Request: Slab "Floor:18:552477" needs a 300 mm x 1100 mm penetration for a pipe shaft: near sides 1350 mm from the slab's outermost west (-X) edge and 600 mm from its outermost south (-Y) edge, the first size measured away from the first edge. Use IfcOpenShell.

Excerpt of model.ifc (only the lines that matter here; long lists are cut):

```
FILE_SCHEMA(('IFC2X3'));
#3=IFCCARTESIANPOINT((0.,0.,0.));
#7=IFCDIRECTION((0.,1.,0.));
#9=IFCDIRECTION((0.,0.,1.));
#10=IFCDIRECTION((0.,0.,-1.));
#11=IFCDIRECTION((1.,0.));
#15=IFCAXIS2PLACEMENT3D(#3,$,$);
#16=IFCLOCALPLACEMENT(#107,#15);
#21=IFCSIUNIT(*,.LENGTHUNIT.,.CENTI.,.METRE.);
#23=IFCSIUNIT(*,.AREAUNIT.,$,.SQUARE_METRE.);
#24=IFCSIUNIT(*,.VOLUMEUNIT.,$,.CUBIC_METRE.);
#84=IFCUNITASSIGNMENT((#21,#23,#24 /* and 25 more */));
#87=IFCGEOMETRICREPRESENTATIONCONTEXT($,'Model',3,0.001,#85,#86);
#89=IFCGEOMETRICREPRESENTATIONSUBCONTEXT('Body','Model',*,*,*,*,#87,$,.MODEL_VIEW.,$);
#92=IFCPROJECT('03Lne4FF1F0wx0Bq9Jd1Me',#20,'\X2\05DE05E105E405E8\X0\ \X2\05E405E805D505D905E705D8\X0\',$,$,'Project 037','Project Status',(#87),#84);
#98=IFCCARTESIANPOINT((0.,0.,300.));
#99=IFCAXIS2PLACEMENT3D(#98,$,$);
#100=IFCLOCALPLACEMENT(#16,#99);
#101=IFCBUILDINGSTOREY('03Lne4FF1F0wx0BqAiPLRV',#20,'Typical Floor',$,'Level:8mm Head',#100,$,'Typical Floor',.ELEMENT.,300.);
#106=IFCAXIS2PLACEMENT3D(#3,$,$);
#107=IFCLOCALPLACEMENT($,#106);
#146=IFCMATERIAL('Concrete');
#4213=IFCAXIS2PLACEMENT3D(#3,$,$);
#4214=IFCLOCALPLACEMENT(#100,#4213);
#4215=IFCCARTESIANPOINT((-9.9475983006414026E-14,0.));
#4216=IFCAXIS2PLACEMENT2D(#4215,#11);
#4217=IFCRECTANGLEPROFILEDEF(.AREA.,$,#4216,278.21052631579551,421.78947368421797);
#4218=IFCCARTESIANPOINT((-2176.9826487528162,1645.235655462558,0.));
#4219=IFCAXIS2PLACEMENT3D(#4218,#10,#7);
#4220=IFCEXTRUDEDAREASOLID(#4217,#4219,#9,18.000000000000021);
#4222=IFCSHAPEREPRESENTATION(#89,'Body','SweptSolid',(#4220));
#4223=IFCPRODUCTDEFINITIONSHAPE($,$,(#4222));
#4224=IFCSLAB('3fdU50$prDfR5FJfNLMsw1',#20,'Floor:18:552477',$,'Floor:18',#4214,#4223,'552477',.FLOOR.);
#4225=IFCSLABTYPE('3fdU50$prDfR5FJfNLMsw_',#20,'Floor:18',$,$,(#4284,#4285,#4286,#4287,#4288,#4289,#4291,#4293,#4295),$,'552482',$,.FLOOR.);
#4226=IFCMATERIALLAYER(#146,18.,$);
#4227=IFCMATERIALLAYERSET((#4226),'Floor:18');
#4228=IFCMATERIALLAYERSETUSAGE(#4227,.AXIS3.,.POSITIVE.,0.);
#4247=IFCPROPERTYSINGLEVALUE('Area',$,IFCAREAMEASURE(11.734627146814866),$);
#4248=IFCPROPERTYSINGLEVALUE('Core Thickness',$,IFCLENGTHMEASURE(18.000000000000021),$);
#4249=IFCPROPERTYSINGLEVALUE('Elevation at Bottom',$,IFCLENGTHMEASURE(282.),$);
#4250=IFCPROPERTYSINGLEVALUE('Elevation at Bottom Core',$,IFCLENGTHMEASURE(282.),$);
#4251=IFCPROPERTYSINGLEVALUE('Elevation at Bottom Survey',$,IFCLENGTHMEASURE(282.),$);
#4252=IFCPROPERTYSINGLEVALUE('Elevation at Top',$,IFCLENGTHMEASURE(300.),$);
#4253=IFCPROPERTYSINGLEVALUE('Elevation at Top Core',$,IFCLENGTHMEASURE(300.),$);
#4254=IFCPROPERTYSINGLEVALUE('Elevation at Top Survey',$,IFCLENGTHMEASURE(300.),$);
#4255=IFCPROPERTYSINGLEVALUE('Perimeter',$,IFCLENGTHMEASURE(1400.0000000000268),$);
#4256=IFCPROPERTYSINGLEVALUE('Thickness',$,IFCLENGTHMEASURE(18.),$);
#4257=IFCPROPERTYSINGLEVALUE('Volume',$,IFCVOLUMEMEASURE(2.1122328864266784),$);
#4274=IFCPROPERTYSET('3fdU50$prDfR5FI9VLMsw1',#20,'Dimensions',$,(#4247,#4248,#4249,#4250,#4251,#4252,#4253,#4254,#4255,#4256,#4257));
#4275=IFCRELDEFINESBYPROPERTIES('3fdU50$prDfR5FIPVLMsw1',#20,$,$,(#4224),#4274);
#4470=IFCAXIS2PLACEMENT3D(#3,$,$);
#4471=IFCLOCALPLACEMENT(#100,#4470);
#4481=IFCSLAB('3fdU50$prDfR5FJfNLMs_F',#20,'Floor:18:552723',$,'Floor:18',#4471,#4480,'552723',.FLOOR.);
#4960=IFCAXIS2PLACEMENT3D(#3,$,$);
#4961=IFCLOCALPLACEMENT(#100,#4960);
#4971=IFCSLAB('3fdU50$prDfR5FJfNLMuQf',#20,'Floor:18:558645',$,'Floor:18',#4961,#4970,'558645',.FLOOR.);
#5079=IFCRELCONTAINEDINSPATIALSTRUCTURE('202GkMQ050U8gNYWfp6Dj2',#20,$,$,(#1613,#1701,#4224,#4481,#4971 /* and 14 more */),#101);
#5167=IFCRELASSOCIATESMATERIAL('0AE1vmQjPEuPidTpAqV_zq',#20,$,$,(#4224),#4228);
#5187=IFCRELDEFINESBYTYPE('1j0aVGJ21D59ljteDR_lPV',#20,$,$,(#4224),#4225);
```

```python
import numpy as np
import ifcopenshell
import ifcopenshell.api.feature
import ifcopenshell.api.geometry
import ifcopenshell.api.pset
import ifcopenshell.api.root
import ifcopenshell.geom
import ifcopenshell.util.element
import ifcopenshell.util.placement
import ifcopenshell.util.representation
import ifcopenshell.util.shape
import ifcopenshell.util.unit

model = ifcopenshell.open("model.ifc")
unit_scale = ifcopenshell.util.unit.calculate_unit_scale(model)
area_scale = ifcopenshell.util.unit.calculate_unit_scale(model, "AREAUNIT")
volume_scale = ifcopenshell.util.unit.calculate_unit_scale(model, "VOLUMEUNIT")
settings = ifcopenshell.geom.settings()


def volume(element):
    """Net volume in cubic metres, openings subtracted."""
    shape = ifcopenshell.geom.create_shape(settings, element)
    return ifcopenshell.util.shape.get_volume(shape.geometry)


slab = model.by_id(4224)
before = volume(slab)

# Extent in the slab's own axes, in metres. The edges named are its -X and -Y sides.
slab_shape = ifcopenshell.geom.create_shape(settings, slab)
vertices = ifcopenshell.util.shape.get_vertices(slab_shape.geometry)
x_min, y_min, bottom = vertices.min(axis=0)
top = vertices[:, 2].max()

opening = ifcopenshell.api.root.create_entity(model, ifc_class="IfcOpeningElement", name="Pipe shaft opening")
context = ifcopenshell.util.representation.get_context(model, "Model", "Body", "MODEL_VIEW")
width, depth = 0.3, 1.1
outline = [(0.0, 0.0), (width, 0.0), (width, depth), (0.0, depth), (0.0, 0.0)]
# Overshoot both faces by 50 mm so the cut is clean.
shape = ifcopenshell.api.geometry.add_slab_representation(
    model, context=context, depth=top - bottom + 0.1, polyline=outline
)
ifcopenshell.api.geometry.assign_representation(model, product=opening, representation=shape)

matrix = ifcopenshell.util.placement.get_local_placement(slab.ObjectPlacement)
matrix[:, 3] = matrix @ np.append(np.array([x_min + 1.35, y_min + 0.6, bottom - 0.05]) / unit_scale, 1.0)
ifcopenshell.api.geometry.edit_object_placement(model, product=opening, matrix=matrix, is_si=False)
ifcopenshell.api.feature.add_feature(model, feature=opening, element=slab)

after = volume(slab)

# Update the slab's stored quantities.
pset = model.by_id(ifcopenshell.util.element.get_pset(slab, "Dimensions", should_inherit=False)["id"])
ifcopenshell.api.pset.edit_pset(model, pset=pset, properties={
    "Area": model.create_entity("IfcAreaMeasure", after / (top - bottom) / area_scale),
    "Volume": model.create_entity("IfcVolumeMeasure", after / volume_scale),
})

print(f"slab volume {before:.3f} -> {after:.3f} m3")

model.write("model_rev.ifc")
```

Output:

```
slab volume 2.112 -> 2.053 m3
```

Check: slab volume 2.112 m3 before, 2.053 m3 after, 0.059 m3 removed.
